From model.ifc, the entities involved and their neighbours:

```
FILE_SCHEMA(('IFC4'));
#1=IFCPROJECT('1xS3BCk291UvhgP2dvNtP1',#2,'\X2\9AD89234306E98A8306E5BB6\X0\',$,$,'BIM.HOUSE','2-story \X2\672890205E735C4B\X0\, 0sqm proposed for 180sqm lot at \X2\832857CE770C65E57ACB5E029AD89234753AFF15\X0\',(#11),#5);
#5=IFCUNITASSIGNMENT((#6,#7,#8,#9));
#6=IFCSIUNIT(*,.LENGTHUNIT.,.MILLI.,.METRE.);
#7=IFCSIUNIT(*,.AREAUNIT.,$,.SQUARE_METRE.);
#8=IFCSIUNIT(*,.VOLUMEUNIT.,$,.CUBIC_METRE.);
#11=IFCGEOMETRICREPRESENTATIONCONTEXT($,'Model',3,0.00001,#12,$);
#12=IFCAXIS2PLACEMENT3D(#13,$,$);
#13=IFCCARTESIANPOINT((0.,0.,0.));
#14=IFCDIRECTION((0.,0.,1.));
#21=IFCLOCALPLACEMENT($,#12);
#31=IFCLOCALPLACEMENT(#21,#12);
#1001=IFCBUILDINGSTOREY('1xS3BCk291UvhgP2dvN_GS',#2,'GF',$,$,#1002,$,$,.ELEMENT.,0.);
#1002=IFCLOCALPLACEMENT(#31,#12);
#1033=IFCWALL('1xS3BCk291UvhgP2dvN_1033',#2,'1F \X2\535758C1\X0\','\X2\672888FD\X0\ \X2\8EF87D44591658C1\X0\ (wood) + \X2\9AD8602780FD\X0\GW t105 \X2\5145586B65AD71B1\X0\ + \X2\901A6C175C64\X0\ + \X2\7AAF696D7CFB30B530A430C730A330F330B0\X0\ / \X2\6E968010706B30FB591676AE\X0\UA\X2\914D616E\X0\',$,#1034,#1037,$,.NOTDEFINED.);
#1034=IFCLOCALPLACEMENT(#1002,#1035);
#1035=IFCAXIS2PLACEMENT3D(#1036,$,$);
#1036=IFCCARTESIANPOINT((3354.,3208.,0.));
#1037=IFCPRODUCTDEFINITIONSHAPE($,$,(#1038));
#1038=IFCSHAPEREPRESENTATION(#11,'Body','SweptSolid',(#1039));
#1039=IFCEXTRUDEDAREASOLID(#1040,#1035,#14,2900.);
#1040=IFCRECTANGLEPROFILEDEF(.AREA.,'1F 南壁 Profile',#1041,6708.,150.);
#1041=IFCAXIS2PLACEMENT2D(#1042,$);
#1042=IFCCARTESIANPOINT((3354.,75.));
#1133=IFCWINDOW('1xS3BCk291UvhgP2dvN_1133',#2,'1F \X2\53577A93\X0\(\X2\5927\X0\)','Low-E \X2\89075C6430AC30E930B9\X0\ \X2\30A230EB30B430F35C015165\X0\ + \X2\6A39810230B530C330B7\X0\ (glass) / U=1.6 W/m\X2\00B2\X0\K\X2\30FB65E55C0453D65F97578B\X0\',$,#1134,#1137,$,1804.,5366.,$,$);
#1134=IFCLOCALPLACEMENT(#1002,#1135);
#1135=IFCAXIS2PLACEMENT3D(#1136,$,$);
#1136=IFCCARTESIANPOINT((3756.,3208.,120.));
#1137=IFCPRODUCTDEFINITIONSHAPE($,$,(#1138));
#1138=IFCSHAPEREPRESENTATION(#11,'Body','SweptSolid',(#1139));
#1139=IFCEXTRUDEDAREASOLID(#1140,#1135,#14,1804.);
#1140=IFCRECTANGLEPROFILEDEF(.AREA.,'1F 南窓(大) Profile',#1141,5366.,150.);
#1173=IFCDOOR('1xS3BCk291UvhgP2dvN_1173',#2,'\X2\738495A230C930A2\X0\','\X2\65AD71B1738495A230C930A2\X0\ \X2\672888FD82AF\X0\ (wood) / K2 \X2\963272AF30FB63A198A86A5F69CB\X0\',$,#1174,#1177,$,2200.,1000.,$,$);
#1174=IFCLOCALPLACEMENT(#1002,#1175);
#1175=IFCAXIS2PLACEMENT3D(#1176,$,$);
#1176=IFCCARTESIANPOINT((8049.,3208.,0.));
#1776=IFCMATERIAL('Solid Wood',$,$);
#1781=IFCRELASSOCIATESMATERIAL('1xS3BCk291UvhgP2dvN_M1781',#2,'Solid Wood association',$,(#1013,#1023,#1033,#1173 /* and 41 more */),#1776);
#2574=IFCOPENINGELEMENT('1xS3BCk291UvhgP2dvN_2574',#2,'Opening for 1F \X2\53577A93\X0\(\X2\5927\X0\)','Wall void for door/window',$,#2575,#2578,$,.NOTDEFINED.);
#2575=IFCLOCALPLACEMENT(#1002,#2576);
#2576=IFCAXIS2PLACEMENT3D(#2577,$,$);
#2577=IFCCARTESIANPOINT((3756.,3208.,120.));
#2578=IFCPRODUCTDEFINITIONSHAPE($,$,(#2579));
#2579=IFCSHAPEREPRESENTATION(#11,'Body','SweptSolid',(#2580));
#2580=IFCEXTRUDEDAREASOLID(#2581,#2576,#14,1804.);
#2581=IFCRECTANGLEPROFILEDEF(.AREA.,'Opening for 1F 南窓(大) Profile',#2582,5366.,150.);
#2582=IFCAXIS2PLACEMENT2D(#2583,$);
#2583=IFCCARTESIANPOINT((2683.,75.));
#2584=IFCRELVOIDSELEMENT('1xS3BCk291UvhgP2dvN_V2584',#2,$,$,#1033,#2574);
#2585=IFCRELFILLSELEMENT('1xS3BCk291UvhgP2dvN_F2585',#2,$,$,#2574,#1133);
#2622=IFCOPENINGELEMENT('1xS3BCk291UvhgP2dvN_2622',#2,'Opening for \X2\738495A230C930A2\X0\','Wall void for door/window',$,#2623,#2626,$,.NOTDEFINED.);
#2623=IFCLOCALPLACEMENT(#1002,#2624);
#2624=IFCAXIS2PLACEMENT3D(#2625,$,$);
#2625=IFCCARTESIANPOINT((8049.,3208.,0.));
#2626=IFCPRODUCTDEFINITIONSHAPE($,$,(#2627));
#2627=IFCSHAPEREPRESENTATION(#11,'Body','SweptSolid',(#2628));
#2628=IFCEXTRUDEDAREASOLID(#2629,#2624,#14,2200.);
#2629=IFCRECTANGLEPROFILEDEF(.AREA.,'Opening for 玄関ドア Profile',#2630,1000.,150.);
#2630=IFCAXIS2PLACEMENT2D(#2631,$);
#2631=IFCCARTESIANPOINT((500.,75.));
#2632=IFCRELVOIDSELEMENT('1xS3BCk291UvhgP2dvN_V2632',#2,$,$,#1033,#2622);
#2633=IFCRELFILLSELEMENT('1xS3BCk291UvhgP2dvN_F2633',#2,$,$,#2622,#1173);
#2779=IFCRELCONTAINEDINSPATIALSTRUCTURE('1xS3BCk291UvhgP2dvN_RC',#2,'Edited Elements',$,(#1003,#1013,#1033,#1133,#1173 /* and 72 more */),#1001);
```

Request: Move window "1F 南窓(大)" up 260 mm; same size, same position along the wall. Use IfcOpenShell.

```python
import numpy as np
import ifcopenshell
import ifcopenshell.api.geometry
import ifcopenshell.util.placement
import ifcopenshell.util.unit

model = ifcopenshell.open("model.ifc")
unit_scale = ifcopenshell.util.unit.calculate_unit_scale(model)

window = model.by_id(1133)
opening = window.FillsVoids[0].RelatingOpeningElement
dz = 260.0

shift = np.array([0.0, 0.0, dz])
# The window is not placed relative to its opening, so move both.
for product in (opening, window):
    matrix = ifcopenshell.util.placement.get_local_placement(product.ObjectPlacement)
    matrix[:3, 3] += shift
    ifcopenshell.api.geometry.edit_object_placement(model, product=product, matrix=matrix, is_si=False)

print(f"moved by {dz * unit_scale:+.3f} m")

model.write("model_rev.ifc")
```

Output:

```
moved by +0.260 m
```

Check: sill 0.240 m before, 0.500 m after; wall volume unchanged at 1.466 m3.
